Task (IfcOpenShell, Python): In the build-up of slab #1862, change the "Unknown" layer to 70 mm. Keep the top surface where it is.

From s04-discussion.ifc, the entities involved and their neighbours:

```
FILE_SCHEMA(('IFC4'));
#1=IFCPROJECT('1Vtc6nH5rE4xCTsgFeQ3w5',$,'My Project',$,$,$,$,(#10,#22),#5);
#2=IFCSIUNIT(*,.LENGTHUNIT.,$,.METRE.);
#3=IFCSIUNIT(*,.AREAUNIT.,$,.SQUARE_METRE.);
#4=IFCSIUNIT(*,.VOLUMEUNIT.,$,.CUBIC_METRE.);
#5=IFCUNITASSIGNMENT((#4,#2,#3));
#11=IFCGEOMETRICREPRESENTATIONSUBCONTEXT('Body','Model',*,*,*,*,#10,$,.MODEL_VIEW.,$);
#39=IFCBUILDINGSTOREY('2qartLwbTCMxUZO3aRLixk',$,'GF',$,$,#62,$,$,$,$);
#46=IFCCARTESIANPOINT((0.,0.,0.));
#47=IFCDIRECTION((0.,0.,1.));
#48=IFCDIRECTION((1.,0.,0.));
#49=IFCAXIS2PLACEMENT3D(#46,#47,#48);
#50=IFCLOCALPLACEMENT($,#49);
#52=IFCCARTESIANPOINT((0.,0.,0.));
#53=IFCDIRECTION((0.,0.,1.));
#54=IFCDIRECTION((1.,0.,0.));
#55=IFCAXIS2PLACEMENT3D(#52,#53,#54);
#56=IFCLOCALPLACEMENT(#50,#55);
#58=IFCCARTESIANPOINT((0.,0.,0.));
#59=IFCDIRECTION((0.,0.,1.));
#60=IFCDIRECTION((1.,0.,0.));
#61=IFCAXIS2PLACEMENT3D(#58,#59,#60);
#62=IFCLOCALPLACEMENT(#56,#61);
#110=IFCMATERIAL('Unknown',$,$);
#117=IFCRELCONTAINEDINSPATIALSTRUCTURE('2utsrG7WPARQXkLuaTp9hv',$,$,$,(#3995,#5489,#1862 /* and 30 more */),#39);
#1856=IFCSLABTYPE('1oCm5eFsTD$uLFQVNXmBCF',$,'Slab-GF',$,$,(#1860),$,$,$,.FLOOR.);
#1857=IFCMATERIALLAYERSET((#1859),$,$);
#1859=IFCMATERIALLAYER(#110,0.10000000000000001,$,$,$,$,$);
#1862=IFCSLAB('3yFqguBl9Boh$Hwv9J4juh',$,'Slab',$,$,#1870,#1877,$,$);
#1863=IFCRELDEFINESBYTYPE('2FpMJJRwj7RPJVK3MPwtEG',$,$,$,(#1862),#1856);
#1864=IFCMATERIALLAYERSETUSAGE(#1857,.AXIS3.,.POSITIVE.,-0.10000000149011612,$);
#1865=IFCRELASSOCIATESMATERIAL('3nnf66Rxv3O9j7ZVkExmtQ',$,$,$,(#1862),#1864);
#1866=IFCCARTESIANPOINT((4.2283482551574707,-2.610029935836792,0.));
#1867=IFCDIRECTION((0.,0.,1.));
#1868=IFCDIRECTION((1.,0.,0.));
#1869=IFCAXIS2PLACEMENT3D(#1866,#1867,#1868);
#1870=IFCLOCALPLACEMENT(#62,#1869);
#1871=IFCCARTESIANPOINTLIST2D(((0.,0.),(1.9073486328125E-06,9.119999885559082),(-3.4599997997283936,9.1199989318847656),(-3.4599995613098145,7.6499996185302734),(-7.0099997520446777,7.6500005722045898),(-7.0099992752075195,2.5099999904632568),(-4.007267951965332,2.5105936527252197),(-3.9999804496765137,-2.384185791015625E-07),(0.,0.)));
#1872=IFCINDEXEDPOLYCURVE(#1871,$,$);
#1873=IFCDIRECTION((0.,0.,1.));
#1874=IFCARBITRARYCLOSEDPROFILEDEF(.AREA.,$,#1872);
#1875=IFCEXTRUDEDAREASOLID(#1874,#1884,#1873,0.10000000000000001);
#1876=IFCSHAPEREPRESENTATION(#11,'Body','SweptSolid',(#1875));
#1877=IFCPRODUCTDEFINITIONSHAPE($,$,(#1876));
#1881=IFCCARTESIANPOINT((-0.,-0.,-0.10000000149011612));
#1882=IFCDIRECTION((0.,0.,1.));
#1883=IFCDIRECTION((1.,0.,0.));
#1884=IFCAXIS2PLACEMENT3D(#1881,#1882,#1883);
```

```python
import ifcopenshell
import ifcopenshell.util.element
import ifcopenshell.util.representation
import ifcopenshell.util.unit

model = ifcopenshell.open("s04-discussion.ifc")
unit_scale = ifcopenshell.util.unit.calculate_unit_scale(model)

layer_set = model.by_id(1857)
layer = next(l for l in layer_set.MaterialLayers if l.Material and l.Material.Name == "Unknown")
change = 0.07 / unit_scale - layer.LayerThickness
layer.LayerThickness += change

# Geometry does not follow the layer set by itself.
slabs = [e for e in ifcopenshell.util.element.get_elements_by_material(model, layer_set) if e.is_a("IfcSlab")]
for slab in sorted(slabs, key=lambda e: e.id()):
    body = ifcopenshell.util.representation.get_representation(slab, "Model", "Body")
    solid = body.Items[0]
    old_depth = solid.Depth
    solid.Depth += change
    # Extruded upwards: lower the start of the extrusion so the top stays.
    x, y, z = solid.Position.Location.Coordinates
    solid.Position.Location = model.createIfcCartesianPoint((x, y, z - change))
    print(slab.id(), f"{old_depth:g} -> {solid.Depth:g}")

# The layers are counted up from the underside, which has moved.
for usage in {ifcopenshell.util.element.get_material(slab) for slab in slabs}:
    usage.OffsetFromReferenceLine -= change

model.write("s04-discussion-out.ifc")
```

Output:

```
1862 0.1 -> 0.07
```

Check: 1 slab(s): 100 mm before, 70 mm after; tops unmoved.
